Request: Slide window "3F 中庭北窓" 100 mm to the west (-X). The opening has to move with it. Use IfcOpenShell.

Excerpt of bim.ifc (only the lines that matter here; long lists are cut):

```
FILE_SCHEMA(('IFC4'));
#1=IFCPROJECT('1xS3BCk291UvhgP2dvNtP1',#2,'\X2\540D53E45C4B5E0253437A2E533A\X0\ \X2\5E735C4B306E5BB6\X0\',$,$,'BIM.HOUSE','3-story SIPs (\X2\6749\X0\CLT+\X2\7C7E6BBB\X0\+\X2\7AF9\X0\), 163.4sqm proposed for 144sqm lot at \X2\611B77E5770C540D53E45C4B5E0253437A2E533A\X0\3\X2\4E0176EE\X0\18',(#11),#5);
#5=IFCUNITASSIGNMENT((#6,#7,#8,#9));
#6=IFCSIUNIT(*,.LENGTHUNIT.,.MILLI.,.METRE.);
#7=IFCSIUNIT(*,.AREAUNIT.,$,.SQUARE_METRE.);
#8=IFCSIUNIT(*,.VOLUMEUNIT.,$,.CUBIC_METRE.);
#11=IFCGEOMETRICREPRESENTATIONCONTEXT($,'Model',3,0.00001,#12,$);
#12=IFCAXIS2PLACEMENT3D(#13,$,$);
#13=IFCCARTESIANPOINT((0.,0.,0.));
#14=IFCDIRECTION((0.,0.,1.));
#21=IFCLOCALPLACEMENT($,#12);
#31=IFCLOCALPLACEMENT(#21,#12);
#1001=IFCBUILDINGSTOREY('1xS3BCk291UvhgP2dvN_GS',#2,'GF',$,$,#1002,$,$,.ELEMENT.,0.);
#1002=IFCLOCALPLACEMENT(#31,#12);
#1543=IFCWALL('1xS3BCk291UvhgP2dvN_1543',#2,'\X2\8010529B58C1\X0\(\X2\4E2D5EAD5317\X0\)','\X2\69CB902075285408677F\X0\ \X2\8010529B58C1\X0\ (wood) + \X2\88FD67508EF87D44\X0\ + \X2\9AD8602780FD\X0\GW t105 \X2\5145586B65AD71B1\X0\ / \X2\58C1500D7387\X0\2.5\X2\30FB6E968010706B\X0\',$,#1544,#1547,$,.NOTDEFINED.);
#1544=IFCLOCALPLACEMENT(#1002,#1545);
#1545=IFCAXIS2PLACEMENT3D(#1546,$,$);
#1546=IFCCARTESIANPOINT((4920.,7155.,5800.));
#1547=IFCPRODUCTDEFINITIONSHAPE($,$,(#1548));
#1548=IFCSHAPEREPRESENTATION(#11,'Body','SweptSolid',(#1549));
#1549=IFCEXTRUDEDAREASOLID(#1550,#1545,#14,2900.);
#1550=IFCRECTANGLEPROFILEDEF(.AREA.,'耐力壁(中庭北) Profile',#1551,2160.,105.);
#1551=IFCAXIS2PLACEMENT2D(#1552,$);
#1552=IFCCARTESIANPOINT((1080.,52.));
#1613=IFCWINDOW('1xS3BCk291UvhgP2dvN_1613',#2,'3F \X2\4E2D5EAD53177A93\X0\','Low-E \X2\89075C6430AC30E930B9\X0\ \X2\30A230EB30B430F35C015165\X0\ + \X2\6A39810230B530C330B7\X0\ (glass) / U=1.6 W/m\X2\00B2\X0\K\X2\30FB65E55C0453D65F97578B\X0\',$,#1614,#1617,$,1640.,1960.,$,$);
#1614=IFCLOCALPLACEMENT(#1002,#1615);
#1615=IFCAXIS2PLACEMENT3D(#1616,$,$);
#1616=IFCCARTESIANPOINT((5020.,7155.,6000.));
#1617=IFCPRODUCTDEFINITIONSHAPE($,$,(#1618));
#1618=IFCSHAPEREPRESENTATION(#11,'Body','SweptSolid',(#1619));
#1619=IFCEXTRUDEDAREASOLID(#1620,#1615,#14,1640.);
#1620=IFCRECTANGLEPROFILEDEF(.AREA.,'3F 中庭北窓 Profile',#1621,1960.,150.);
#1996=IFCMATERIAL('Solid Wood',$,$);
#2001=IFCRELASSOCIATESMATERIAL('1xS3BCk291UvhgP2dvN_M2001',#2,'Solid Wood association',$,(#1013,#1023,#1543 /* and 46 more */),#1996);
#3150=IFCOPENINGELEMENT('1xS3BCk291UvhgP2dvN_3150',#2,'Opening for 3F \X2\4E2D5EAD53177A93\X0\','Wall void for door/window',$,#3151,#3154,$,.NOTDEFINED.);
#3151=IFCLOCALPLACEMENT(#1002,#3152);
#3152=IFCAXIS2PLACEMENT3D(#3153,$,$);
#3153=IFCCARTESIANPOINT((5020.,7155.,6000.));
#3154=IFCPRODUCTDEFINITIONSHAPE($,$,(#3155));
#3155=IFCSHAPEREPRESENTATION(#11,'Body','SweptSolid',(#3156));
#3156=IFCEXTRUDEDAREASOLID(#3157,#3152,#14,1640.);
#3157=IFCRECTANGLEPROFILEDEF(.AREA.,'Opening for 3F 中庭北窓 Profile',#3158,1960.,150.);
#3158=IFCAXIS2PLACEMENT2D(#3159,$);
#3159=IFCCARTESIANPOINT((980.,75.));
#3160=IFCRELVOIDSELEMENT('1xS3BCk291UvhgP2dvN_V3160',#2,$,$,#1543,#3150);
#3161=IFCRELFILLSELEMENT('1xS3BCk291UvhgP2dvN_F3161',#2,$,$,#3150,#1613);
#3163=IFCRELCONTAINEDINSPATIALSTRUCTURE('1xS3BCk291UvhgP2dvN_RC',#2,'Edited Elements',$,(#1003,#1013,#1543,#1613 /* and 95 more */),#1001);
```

```python
import ifcopenshell
import ifcopenshell.api.geometry
import ifcopenshell.util.placement

model = ifcopenshell.open("bim.ifc")

window = model.by_id(1613)
opening = window.FillsVoids[0].RelatingOpeningElement
wall = opening.VoidsElements[0].RelatingBuildingElement

wall_matrix = ifcopenshell.util.placement.get_local_placement(wall.ObjectPlacement)
shift = wall_matrix[:3, 0] * -100.0
before = ifcopenshell.util.placement.get_local_placement(window.ObjectPlacement)[:3, 3].copy()

# The window is not placed relative to its opening, so move both.
for product in (opening, window):
    matrix = ifcopenshell.util.placement.get_local_placement(product.ObjectPlacement)
    matrix[:3, 3] += shift
    ifcopenshell.api.geometry.edit_object_placement(model, product=product, matrix=matrix, is_si=False)

after = ifcopenshell.util.placement.get_local_placement(window.ObjectPlacement)[:3, 3]
print("window moved by", (after - before).round(3) + 0.0)

model.write("bim_v2.ifc")
```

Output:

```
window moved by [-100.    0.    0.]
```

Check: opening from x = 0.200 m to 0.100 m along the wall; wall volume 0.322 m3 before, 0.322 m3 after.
